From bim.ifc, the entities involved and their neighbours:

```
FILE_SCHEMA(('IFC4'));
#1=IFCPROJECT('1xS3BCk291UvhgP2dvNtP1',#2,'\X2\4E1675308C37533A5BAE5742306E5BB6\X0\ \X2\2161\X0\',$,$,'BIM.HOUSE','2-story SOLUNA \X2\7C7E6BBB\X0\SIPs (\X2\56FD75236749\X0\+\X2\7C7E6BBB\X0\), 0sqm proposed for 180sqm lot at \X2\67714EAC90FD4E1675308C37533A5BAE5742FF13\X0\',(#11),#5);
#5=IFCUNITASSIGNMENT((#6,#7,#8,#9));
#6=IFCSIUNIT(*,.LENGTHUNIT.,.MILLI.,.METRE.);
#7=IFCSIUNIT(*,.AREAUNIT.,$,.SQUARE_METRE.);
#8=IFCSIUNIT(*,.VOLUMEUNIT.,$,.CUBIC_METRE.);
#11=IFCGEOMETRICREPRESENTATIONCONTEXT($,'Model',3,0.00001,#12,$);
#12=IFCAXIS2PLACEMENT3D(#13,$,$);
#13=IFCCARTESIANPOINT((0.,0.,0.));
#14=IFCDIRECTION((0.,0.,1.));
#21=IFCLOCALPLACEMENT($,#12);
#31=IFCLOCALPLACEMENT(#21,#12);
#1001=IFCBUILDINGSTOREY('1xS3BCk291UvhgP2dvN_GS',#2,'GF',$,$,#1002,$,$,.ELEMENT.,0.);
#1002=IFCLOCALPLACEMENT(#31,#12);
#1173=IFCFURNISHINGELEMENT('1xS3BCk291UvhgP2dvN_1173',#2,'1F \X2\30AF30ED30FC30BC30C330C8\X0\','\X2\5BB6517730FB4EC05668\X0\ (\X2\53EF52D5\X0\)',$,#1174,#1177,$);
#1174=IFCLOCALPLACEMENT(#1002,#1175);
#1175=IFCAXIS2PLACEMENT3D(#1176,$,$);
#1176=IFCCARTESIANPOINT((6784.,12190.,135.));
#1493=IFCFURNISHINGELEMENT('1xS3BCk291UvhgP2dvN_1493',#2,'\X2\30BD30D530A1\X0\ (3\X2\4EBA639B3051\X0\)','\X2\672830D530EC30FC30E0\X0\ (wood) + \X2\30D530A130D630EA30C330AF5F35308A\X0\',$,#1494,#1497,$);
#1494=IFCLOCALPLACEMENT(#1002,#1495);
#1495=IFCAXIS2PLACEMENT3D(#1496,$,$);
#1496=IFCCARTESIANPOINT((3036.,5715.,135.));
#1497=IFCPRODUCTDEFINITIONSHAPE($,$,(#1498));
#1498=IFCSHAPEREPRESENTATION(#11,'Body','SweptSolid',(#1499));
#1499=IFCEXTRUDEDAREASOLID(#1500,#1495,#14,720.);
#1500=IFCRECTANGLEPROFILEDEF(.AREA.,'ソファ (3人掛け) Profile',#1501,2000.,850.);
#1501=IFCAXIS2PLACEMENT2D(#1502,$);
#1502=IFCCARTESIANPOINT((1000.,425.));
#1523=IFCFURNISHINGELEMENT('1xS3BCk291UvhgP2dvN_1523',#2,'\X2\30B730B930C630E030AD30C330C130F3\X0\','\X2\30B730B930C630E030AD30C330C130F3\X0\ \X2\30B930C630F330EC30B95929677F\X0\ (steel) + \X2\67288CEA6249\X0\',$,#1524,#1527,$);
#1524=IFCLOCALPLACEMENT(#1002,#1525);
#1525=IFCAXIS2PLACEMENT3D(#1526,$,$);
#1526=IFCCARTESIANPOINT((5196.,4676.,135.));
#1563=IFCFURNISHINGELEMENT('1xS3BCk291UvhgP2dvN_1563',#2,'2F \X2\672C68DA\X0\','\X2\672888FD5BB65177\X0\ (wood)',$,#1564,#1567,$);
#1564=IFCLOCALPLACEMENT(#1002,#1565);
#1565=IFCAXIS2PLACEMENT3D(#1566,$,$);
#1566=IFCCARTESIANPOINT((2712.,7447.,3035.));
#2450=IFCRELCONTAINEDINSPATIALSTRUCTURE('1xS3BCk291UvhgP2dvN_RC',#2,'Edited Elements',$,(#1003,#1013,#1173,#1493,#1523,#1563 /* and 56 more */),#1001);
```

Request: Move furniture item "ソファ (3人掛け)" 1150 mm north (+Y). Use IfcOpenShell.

```python
import ifcopenshell
import ifcopenshell.api.geometry
import ifcopenshell.util.placement

model = ifcopenshell.open("bim.ifc")

item = model.by_guid("1xS3BCk291UvhgP2dvN_1493")
matrix = ifcopenshell.util.placement.get_local_placement(item.ObjectPlacement)
matrix[1, 3] += 1150.0
ifcopenshell.api.geometry.edit_object_placement(model, product=item, matrix=matrix, is_si=False)

print(ifcopenshell.util.placement.get_local_placement(item.ObjectPlacement).round(3) + 0.0)

model.write("bim_rev.ifc")
```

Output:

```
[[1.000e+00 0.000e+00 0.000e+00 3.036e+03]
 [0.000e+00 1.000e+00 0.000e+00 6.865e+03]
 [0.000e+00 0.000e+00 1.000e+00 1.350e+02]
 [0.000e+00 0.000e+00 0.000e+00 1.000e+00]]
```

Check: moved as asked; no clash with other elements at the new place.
